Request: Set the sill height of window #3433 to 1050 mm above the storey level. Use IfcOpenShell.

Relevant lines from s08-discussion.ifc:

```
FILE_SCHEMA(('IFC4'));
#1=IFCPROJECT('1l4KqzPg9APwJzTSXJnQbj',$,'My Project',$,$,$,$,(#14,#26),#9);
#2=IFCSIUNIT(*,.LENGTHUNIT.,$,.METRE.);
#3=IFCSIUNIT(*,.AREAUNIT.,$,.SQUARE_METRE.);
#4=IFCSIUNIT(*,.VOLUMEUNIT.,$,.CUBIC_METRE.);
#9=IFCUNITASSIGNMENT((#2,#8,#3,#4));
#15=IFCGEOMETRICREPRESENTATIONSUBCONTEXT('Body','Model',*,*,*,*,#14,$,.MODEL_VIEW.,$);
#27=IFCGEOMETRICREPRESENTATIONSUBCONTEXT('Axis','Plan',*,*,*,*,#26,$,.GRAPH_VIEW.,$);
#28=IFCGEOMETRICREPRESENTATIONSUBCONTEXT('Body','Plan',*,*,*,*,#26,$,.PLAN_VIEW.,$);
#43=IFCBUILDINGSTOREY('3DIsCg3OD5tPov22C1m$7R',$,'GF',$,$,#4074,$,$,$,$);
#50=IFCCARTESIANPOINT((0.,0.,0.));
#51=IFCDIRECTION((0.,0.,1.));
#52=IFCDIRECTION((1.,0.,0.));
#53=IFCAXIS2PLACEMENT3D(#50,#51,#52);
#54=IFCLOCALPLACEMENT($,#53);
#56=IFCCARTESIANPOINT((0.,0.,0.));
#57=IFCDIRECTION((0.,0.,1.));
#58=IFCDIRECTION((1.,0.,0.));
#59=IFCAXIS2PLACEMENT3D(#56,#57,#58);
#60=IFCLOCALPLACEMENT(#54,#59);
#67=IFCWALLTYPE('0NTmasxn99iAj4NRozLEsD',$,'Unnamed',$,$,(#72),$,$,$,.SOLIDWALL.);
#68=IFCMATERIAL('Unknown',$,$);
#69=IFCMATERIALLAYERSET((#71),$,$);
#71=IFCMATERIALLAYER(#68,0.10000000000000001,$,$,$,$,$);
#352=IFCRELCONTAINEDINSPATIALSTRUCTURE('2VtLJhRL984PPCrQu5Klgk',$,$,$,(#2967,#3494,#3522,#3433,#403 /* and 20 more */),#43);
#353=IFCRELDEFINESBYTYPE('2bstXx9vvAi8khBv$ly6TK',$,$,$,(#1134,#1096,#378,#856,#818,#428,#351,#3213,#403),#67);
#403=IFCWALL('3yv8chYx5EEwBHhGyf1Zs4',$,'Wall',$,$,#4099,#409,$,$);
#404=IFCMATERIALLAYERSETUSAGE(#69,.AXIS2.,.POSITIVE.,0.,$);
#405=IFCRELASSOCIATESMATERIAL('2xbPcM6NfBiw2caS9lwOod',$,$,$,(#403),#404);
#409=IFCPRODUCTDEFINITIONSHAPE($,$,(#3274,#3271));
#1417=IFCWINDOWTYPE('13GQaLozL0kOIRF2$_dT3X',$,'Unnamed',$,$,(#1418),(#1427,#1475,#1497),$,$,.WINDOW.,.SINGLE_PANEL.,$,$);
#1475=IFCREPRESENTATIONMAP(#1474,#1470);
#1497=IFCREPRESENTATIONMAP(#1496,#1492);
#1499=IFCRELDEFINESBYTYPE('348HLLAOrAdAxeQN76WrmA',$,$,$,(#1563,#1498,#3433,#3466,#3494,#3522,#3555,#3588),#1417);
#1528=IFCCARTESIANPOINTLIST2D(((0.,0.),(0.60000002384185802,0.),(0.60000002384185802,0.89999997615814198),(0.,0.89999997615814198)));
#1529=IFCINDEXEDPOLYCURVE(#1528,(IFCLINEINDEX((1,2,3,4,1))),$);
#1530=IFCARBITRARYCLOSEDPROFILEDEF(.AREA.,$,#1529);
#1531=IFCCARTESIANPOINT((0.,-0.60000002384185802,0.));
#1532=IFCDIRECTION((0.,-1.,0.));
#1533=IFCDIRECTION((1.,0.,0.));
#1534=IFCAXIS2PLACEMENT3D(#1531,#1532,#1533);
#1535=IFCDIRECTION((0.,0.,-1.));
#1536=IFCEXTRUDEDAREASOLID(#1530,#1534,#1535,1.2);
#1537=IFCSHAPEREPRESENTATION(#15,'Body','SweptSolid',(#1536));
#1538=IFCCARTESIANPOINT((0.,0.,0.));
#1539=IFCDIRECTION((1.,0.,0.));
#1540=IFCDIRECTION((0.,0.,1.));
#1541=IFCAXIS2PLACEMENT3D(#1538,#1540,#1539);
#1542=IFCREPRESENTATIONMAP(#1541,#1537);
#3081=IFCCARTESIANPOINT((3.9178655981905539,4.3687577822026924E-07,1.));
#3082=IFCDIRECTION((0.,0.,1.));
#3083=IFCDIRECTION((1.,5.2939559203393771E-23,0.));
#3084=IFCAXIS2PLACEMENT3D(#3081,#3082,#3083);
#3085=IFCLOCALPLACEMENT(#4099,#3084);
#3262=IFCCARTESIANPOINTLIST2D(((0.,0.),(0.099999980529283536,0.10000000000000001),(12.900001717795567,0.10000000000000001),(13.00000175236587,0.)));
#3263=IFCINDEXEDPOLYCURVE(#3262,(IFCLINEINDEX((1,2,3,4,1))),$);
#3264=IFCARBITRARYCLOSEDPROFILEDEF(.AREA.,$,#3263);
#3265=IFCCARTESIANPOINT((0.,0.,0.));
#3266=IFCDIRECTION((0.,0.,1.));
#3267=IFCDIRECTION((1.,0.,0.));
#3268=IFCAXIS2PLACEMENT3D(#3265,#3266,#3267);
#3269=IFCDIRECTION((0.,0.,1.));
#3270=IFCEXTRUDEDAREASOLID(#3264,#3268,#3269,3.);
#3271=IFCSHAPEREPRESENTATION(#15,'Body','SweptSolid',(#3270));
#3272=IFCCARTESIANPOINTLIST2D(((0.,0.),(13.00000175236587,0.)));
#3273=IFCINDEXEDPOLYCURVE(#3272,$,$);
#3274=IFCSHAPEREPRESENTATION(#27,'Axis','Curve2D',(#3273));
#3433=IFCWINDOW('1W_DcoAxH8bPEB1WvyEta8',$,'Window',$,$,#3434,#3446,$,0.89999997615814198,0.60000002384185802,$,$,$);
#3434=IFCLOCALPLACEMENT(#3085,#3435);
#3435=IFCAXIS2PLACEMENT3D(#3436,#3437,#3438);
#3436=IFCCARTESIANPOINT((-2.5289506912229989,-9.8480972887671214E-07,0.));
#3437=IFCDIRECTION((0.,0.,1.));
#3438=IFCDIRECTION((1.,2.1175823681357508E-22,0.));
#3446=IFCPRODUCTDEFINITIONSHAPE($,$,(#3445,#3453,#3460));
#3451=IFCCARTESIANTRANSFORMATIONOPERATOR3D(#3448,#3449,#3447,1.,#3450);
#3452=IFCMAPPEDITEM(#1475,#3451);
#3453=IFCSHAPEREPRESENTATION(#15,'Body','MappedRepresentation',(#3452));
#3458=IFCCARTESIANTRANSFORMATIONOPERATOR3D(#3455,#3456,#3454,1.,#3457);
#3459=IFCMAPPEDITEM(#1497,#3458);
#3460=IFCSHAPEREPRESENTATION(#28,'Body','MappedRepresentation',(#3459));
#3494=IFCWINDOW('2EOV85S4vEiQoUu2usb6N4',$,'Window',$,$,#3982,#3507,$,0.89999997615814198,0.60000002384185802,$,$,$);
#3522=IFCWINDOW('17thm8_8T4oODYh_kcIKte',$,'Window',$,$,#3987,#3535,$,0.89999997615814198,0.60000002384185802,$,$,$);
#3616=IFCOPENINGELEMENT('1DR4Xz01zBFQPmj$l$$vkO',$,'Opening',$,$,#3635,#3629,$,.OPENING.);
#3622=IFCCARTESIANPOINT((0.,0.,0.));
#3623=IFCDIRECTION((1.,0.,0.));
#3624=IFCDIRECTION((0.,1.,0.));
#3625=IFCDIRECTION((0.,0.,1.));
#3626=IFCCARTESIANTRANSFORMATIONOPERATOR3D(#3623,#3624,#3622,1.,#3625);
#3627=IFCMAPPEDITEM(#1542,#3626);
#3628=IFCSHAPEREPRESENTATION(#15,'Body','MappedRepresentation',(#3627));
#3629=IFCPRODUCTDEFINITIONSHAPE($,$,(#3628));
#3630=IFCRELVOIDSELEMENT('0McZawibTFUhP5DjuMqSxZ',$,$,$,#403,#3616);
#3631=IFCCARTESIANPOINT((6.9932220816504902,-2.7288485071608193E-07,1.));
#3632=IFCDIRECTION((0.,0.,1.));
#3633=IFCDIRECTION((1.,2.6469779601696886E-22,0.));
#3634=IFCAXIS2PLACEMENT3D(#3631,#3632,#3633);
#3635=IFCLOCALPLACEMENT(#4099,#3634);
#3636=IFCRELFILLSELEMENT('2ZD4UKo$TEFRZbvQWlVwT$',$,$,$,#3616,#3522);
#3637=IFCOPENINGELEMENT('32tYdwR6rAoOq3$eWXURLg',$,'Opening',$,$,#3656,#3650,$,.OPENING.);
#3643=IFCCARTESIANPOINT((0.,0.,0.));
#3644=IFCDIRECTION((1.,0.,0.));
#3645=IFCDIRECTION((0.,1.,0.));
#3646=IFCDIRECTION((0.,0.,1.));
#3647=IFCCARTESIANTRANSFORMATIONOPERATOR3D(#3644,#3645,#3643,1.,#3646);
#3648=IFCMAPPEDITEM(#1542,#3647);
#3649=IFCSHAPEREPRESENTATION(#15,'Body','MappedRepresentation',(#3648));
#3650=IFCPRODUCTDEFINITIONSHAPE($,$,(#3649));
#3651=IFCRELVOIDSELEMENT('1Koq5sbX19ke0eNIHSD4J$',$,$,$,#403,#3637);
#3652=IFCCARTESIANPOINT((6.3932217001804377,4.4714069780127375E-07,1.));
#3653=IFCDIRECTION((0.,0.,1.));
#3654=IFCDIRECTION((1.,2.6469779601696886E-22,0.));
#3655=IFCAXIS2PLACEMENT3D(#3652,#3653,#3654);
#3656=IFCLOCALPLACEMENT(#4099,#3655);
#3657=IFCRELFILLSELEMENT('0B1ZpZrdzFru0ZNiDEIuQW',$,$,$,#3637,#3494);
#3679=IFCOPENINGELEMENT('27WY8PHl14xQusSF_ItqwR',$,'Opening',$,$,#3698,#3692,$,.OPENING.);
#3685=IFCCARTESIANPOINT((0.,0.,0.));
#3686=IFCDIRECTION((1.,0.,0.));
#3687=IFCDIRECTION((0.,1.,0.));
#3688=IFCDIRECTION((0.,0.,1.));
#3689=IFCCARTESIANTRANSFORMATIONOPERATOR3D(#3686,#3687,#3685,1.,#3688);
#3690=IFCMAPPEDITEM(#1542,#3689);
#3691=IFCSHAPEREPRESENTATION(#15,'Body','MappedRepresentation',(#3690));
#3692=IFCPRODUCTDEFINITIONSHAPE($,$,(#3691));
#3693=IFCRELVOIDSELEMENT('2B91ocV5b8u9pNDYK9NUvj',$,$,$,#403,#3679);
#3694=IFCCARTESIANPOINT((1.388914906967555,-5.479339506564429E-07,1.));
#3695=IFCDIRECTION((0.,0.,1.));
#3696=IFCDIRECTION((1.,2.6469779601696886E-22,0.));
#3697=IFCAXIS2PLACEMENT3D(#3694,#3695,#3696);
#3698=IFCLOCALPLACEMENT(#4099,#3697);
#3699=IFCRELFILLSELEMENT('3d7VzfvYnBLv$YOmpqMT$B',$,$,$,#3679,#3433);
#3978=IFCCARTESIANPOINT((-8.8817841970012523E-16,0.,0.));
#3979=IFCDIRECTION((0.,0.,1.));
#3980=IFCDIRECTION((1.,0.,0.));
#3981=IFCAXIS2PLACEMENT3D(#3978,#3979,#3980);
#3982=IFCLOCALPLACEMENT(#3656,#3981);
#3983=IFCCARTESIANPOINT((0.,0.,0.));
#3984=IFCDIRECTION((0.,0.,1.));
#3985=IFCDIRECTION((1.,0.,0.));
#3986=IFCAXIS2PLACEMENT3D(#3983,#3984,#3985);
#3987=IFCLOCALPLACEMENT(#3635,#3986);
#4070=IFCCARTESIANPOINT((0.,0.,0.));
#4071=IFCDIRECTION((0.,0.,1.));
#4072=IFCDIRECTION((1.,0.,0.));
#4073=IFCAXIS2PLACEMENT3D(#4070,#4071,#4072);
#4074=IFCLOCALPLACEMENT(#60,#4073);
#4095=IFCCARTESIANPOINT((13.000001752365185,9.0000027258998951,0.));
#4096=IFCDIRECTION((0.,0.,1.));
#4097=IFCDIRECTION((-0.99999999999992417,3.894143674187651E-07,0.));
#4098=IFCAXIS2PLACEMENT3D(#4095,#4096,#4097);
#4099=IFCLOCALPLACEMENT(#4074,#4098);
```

```python
import numpy as np
import ifcopenshell
import ifcopenshell.api.geometry
import ifcopenshell.geom
import ifcopenshell.util.element
import ifcopenshell.util.placement
import ifcopenshell.util.shape
import ifcopenshell.util.unit

model = ifcopenshell.open("s08-discussion.ifc")
unit_scale = ifcopenshell.util.unit.calculate_unit_scale(model)

window = model.by_id(3433)
opening = window.FillsVoids[0].RelatingOpeningElement
storey = ifcopenshell.util.element.get_container(window, ifc_class="IfcBuildingStorey")
level = ifcopenshell.util.placement.get_local_placement(storey.ObjectPlacement)[2, 3]

# The opening's origin need not be at the sill, so measure its lowest point.
shape = ifcopenshell.geom.create_shape(ifcopenshell.geom.settings(), opening)
bottom = ifcopenshell.util.shape.get_shape_bottom_elevation(shape, shape.geometry) / unit_scale
dz = level + 1.05 - bottom

shift = np.array([0.0, 0.0, dz])
# The window is not placed relative to its opening, so move both.
for product in (opening, window):
    matrix = ifcopenshell.util.placement.get_local_placement(product.ObjectPlacement)
    matrix[:3, 3] += shift
    ifcopenshell.api.geometry.edit_object_placement(model, product=product, matrix=matrix, is_si=False)

print(f"moved by {dz * unit_scale:+.3f} m")

model.write("s08-discussion_rev.ifc")
```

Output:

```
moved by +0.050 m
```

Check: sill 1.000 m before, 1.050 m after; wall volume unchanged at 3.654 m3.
